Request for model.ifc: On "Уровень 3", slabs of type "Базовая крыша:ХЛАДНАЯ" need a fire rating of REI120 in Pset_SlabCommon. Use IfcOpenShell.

First a look at what the model holds.

```python
import ifcopenshell
import ifcopenshell.util.element

model = ifcopenshell.open("model.ifc")
print(model.schema)
storey = next(s for s in model.by_type("IfcBuildingStorey") if s.Name == "Уровень 3")
slabs = [e for e in ifcopenshell.util.element.get_decomposition(storey) if e.is_a("IfcSlab")]
seen = {}
for e in slabs:
    element_type = ifcopenshell.util.element.get_type(e)
    key = (element_type.Name if element_type != e and element_type else None, ifcopenshell.util.element.get_pset(e, "Pset_SlabCommon", "FireRating"))
    seen[key] = seen.get(key, 0) + 1
for (name, value), count in sorted(seen.items(), key=str):
    print(count, "x", name, "|", value)
```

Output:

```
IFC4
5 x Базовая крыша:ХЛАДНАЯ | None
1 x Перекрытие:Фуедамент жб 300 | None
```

```python
import ifcopenshell
import ifcopenshell.api.pset
import ifcopenshell.util.element

model = ifcopenshell.open("model.ifc")

storey = next(s for s in model.by_type("IfcBuildingStorey") if s.Name == "Уровень 3")
slabs = [e for e in ifcopenshell.util.element.get_decomposition(storey) if e.is_a("IfcSlab")]

count = 0
for e in slabs:
    element_type = ifcopenshell.util.element.get_type(e)
    if element_type in (None, e) or element_type.Name != "Базовая крыша:ХЛАДНАЯ":
        continue
    # add_pset returns the element's existing set when there is one.
    pset = ifcopenshell.api.pset.add_pset(model, product=e, name="Pset_SlabCommon")
    ifcopenshell.api.pset.edit_pset(model, pset=pset, properties={"FireRating": "REI120"})
    count += 1

print(count, "slabs updated")

model.write("model-out.ifc")
```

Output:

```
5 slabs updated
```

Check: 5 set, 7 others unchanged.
